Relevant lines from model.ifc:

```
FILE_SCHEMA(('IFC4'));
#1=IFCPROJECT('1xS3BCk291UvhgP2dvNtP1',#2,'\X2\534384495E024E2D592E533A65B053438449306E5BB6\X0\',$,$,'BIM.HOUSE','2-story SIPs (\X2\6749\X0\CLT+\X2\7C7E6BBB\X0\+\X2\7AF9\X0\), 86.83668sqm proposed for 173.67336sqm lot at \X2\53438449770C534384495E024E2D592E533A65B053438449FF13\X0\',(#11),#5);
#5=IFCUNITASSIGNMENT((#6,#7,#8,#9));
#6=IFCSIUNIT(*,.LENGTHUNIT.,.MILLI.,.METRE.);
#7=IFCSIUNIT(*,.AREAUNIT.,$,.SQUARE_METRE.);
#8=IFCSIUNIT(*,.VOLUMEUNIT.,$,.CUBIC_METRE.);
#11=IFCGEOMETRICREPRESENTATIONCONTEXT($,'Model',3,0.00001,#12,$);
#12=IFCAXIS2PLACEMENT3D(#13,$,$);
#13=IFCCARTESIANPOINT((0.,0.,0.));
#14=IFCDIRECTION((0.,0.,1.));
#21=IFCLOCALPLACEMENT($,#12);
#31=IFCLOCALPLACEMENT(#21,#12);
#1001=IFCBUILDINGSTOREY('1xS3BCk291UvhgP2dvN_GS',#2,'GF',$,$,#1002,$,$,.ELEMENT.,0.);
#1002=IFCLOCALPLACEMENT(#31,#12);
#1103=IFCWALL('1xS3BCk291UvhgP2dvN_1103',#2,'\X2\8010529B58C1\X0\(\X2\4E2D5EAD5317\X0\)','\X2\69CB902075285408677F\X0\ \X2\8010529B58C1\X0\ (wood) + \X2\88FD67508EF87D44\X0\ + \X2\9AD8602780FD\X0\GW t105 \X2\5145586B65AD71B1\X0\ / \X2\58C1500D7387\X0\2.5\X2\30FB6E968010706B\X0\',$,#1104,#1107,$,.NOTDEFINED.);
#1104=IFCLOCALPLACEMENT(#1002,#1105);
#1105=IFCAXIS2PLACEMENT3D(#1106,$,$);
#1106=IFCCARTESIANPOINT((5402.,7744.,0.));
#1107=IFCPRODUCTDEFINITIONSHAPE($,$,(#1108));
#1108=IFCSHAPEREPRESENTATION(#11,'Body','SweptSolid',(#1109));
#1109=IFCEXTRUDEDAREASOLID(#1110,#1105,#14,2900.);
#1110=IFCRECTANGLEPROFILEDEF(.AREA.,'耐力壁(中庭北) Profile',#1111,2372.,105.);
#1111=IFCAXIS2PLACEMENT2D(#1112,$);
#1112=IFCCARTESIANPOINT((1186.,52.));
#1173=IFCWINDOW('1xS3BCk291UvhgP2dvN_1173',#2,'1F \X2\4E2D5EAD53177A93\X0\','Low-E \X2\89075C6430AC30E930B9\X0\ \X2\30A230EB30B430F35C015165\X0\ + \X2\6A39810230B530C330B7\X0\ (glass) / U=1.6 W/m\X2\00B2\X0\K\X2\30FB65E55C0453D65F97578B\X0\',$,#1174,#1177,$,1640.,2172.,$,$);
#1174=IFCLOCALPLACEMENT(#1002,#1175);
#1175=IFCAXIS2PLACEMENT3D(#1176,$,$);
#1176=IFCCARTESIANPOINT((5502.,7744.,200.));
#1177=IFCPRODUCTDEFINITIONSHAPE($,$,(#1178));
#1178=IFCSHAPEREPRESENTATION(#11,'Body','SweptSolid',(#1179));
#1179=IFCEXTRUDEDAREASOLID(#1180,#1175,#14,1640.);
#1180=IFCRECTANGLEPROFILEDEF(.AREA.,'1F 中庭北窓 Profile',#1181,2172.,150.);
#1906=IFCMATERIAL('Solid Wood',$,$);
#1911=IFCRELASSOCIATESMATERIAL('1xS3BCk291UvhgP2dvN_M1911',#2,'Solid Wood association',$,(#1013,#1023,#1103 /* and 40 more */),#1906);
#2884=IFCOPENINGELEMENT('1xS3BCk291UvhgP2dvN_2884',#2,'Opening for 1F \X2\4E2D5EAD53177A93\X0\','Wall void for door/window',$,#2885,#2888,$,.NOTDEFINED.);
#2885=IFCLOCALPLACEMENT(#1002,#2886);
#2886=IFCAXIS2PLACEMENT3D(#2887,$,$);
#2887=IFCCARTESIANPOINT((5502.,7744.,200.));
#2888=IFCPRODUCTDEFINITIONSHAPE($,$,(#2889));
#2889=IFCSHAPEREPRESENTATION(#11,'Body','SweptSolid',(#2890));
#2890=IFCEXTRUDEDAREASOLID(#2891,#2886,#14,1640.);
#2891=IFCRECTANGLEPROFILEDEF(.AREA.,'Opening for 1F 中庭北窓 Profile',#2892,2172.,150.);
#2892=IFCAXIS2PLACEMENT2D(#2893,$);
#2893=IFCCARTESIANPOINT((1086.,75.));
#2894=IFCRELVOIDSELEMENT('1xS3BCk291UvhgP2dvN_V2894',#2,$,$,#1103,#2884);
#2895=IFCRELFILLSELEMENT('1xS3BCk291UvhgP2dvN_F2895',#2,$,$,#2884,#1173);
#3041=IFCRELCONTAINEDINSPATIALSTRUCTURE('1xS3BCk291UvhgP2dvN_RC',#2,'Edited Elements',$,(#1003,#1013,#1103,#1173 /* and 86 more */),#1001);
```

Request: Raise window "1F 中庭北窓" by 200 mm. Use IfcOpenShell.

```python
import numpy as np
import ifcopenshell
import ifcopenshell.api.geometry
import ifcopenshell.util.placement
import ifcopenshell.util.unit

model = ifcopenshell.open("model.ifc")
unit_scale = ifcopenshell.util.unit.calculate_unit_scale(model)

window = model.by_id(1173)
opening = window.FillsVoids[0].RelatingOpeningElement
dz = 200.0

shift = np.array([0.0, 0.0, dz])
# The window is not placed relative to its opening, so move both.
for product in (opening, window):
    matrix = ifcopenshell.util.placement.get_local_placement(product.ObjectPlacement)
    matrix[:3, 3] += shift
    ifcopenshell.api.geometry.edit_object_placement(model, product=product, matrix=matrix, is_si=False)

print(f"moved by {dz * unit_scale:+.3f} m")

model.write("model_rev.ifc")
```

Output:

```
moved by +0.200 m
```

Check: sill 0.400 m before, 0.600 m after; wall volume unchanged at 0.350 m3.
